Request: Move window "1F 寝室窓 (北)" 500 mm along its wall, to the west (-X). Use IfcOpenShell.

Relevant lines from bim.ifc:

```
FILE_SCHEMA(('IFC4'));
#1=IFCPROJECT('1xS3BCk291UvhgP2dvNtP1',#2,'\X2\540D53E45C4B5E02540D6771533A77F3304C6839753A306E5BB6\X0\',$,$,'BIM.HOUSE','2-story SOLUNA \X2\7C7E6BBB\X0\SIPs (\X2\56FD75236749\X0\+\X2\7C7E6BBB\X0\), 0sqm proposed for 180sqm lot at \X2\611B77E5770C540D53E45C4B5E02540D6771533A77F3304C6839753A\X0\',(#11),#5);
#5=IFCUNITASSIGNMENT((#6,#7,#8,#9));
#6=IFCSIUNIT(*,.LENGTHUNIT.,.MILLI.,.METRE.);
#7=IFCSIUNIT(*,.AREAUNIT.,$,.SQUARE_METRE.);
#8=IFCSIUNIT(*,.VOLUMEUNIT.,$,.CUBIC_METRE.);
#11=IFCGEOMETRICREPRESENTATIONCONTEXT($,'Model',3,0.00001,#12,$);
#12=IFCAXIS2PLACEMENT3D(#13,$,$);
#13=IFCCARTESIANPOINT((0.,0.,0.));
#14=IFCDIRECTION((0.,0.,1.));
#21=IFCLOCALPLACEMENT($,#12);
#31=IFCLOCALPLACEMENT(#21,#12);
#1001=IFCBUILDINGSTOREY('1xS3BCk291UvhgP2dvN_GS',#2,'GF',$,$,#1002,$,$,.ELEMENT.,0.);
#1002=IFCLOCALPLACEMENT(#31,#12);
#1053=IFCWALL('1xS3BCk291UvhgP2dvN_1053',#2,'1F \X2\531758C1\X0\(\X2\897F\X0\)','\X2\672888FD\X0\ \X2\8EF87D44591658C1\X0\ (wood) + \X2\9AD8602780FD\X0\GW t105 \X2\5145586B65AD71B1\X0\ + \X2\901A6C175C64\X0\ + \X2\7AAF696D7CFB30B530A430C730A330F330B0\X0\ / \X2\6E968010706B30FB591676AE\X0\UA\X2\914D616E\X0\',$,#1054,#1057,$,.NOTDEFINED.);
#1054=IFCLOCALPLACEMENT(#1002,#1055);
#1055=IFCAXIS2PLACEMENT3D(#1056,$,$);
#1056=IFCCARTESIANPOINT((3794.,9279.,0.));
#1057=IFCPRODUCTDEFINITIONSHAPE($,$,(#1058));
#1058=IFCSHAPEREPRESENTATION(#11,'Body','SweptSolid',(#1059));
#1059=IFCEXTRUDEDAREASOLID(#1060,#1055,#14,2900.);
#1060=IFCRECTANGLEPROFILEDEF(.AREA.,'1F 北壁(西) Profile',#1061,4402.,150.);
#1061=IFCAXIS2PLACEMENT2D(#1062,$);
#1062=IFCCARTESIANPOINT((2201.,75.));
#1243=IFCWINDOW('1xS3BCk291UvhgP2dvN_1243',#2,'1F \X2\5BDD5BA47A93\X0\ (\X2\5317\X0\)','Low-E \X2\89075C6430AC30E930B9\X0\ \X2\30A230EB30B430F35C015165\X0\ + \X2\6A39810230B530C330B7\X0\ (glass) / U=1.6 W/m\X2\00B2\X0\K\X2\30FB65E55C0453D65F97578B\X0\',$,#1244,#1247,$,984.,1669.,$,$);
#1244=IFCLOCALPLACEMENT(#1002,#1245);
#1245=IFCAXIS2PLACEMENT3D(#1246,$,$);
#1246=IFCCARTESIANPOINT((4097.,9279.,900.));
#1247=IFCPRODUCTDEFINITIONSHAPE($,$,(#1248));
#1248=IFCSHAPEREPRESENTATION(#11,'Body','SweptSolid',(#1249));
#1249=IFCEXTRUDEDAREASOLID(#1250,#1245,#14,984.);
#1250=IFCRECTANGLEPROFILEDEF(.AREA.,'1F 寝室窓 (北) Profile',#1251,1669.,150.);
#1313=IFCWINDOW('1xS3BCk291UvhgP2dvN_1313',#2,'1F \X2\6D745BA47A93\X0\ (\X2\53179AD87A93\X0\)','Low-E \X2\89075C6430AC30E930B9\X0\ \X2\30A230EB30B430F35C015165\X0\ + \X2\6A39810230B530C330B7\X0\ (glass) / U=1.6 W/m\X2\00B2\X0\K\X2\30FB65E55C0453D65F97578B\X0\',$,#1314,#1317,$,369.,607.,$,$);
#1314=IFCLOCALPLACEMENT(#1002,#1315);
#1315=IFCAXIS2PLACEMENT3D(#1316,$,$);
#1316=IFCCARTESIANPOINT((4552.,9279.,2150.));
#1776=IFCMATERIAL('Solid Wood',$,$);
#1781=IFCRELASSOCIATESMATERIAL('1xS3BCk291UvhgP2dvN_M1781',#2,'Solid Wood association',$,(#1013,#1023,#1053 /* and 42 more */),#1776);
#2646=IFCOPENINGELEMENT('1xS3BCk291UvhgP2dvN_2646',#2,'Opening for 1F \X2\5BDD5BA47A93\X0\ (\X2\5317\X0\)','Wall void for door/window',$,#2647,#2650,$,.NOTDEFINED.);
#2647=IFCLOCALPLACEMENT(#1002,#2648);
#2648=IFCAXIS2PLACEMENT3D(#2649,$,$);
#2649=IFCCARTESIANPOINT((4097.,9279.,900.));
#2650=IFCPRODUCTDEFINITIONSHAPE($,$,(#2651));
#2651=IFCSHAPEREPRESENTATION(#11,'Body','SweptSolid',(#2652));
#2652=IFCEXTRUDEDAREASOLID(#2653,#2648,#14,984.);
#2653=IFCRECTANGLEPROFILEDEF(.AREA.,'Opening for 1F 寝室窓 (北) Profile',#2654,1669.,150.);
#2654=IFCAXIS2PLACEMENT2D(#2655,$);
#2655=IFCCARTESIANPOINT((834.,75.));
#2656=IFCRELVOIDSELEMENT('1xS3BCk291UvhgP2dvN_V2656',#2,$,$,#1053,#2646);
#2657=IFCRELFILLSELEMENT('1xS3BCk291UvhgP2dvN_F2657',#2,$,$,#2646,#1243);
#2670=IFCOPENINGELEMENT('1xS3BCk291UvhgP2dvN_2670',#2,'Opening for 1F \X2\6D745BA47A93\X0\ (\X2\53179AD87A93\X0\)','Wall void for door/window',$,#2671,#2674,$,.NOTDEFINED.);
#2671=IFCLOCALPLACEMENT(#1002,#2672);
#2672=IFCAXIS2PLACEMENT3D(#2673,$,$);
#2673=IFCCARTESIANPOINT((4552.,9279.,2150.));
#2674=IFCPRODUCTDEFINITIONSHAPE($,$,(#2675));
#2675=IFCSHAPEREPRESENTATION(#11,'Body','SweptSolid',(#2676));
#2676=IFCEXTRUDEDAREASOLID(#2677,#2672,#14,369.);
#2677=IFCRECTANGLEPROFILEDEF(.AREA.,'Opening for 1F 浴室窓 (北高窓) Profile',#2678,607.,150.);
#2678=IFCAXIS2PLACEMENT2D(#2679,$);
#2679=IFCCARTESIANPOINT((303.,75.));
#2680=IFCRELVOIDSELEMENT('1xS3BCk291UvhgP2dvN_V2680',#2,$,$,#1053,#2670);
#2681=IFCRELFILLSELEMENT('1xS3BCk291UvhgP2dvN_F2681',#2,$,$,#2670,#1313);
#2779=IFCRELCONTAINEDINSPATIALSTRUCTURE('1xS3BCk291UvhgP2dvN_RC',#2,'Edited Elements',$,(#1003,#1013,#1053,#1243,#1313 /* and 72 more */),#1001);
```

```python
import ifcopenshell
import ifcopenshell.api.geometry
import ifcopenshell.util.placement

model = ifcopenshell.open("bim.ifc")

window = model.by_guid("1xS3BCk291UvhgP2dvN_1243")
opening = window.FillsVoids[0].RelatingOpeningElement
wall = opening.VoidsElements[0].RelatingBuildingElement

wall_matrix = ifcopenshell.util.placement.get_local_placement(wall.ObjectPlacement)
shift = wall_matrix[:3, 0] * -500.0
before = ifcopenshell.util.placement.get_local_placement(window.ObjectPlacement)[:3, 3].copy()

# The window is not placed relative to its opening, so move both.
for product in (opening, window):
    matrix = ifcopenshell.util.placement.get_local_placement(product.ObjectPlacement)
    matrix[:3, 3] += shift
    ifcopenshell.api.geometry.edit_object_placement(model, product=product, matrix=matrix, is_si=False)

after = ifcopenshell.util.placement.get_local_placement(window.ObjectPlacement)[:3, 3]
print("window moved by", (after - before).round(3) + 0.0)

model.write("bim_v2.ifc")
```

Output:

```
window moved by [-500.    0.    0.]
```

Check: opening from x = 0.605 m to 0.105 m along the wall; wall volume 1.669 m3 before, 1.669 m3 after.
